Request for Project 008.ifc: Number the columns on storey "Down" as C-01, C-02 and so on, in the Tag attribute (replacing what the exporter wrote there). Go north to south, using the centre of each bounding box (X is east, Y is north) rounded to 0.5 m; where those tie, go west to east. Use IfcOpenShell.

First a look at what the model holds.

```python
import ifcopenshell
import ifcopenshell.util.element
import ifcopenshell.util.placement

model = ifcopenshell.open("Project 008.ifc")
print(model.schema)
storey = next(s for s in model.by_type("IfcBuildingStorey") if s.Name == "Down")
columns = [e for e in ifcopenshell.util.element.get_decomposition(storey) if e.is_a("IfcColumn")]
for e in sorted(columns, key=lambda e: e.id()):
    origin = ifcopenshell.util.placement.get_local_placement(e.ObjectPlacement)[:3, 3]
    print(e.id(), e.Tag, e.Name, origin.round(2) + 0.0, sep=" | ")
```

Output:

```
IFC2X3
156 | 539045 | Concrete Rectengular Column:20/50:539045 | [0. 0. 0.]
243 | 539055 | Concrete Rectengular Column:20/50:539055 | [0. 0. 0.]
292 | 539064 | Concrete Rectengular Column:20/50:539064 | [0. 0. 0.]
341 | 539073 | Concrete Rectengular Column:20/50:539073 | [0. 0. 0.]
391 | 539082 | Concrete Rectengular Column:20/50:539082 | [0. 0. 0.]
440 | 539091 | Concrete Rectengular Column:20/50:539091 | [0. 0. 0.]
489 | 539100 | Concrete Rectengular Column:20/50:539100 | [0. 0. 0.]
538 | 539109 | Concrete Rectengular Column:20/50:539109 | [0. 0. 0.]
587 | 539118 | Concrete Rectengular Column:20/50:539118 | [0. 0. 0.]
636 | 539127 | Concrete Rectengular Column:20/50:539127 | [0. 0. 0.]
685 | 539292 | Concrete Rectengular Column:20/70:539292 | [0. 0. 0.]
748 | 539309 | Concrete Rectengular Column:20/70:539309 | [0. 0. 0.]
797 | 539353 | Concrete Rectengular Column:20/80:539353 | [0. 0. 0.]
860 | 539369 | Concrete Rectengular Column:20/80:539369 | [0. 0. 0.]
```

```python
import ifcopenshell
import ifcopenshell.geom
import ifcopenshell.util.element
import ifcopenshell.util.shape

model = ifcopenshell.open("Project 008.ifc")
settings = ifcopenshell.geom.settings()
settings.set("use-world-coords", True)


def centre(element):
    shape = ifcopenshell.geom.create_shape(settings, element)
    return ifcopenshell.util.shape.get_bbox_centroid(shape.geometry)


storey = next(s for s in model.by_type("IfcBuildingStorey") if s.Name == "Down")
columns = [e for e in ifcopenshell.util.element.get_decomposition(storey) if e.is_a("IfcColumn")]

# Insertion points can sit at a corner or the storey origin, so sort by the geometry (in metres).
centres = {e: centre(e) for e in columns}
columns.sort(key=lambda e: (-round(centres[e][1] / 0.5), centres[e][0]))

for i, e in enumerate(columns, start=1):
    number = f"C-{i:02d}"
    e.Tag = number
    print(e.id(), number)

model.write("Project 008_v2.ifc")
```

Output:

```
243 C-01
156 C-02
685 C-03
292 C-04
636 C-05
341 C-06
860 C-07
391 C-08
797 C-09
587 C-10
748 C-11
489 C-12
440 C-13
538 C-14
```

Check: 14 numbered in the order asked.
